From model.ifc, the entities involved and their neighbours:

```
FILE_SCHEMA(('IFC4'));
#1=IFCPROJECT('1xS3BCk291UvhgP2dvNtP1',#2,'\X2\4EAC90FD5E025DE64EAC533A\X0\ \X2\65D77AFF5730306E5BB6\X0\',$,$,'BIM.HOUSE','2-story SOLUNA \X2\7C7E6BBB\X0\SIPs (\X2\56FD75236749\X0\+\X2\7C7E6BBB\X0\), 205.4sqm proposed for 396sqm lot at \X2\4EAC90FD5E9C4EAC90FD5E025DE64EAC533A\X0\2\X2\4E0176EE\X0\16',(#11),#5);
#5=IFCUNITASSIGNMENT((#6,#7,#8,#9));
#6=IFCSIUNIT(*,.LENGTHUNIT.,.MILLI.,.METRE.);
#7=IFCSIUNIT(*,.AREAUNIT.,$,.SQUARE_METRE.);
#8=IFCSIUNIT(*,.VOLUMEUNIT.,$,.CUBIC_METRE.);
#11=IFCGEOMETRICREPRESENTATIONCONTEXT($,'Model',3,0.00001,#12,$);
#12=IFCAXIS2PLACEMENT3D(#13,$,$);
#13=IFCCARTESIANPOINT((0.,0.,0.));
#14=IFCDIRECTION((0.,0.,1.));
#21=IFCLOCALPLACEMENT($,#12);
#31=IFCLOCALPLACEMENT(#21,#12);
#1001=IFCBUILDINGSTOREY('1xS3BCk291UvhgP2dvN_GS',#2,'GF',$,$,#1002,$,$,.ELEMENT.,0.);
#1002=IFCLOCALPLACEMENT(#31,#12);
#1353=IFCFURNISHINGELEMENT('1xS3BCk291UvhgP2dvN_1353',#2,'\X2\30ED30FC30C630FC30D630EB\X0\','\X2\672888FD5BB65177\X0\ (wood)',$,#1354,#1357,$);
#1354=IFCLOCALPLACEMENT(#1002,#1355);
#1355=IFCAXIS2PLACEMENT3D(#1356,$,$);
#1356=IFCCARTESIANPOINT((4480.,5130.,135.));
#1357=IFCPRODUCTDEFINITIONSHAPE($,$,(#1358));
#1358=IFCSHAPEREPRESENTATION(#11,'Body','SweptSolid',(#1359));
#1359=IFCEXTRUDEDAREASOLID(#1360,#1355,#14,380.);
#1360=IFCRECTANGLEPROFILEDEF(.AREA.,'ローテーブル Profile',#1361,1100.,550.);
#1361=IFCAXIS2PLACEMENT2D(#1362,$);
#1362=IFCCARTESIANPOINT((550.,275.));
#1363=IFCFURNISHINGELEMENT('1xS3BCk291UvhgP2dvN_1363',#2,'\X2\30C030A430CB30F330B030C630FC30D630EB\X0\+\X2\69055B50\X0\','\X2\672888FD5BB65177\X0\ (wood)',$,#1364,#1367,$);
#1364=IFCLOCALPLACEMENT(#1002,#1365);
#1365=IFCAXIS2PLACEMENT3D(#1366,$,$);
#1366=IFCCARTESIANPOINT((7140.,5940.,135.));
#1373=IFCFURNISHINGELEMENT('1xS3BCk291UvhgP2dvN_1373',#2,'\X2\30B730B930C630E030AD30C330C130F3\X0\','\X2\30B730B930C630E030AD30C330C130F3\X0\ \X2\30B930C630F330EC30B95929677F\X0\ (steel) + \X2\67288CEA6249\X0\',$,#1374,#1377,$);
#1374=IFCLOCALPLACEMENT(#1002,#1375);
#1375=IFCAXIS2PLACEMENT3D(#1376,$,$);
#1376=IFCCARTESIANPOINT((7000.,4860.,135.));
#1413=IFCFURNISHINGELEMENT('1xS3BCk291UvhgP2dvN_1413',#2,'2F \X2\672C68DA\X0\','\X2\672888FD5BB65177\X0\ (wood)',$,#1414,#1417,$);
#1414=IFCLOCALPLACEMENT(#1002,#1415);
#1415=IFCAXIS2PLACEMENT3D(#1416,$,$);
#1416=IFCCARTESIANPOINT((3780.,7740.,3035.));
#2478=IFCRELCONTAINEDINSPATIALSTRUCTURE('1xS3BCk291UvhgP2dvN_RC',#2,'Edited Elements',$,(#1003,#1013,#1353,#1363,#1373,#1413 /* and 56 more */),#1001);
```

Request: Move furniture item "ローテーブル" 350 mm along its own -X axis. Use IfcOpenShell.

```python
import ifcopenshell
import ifcopenshell.api.geometry
import ifcopenshell.util.placement

model = ifcopenshell.open("model.ifc")

item = model.by_id(1353)
matrix = ifcopenshell.util.placement.get_local_placement(item.ObjectPlacement)
matrix[:3, 3] -= matrix[:3, 0] * 350.0
ifcopenshell.api.geometry.edit_object_placement(model, product=item, matrix=matrix, is_si=False)

print(ifcopenshell.util.placement.get_local_placement(item.ObjectPlacement).round(3) + 0.0)

model.write("model_edited.ifc")
```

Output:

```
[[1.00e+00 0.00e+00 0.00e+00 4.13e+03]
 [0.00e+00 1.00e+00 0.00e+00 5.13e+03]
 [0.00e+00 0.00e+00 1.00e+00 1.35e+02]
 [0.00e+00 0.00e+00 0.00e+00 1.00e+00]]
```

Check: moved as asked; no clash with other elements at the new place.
